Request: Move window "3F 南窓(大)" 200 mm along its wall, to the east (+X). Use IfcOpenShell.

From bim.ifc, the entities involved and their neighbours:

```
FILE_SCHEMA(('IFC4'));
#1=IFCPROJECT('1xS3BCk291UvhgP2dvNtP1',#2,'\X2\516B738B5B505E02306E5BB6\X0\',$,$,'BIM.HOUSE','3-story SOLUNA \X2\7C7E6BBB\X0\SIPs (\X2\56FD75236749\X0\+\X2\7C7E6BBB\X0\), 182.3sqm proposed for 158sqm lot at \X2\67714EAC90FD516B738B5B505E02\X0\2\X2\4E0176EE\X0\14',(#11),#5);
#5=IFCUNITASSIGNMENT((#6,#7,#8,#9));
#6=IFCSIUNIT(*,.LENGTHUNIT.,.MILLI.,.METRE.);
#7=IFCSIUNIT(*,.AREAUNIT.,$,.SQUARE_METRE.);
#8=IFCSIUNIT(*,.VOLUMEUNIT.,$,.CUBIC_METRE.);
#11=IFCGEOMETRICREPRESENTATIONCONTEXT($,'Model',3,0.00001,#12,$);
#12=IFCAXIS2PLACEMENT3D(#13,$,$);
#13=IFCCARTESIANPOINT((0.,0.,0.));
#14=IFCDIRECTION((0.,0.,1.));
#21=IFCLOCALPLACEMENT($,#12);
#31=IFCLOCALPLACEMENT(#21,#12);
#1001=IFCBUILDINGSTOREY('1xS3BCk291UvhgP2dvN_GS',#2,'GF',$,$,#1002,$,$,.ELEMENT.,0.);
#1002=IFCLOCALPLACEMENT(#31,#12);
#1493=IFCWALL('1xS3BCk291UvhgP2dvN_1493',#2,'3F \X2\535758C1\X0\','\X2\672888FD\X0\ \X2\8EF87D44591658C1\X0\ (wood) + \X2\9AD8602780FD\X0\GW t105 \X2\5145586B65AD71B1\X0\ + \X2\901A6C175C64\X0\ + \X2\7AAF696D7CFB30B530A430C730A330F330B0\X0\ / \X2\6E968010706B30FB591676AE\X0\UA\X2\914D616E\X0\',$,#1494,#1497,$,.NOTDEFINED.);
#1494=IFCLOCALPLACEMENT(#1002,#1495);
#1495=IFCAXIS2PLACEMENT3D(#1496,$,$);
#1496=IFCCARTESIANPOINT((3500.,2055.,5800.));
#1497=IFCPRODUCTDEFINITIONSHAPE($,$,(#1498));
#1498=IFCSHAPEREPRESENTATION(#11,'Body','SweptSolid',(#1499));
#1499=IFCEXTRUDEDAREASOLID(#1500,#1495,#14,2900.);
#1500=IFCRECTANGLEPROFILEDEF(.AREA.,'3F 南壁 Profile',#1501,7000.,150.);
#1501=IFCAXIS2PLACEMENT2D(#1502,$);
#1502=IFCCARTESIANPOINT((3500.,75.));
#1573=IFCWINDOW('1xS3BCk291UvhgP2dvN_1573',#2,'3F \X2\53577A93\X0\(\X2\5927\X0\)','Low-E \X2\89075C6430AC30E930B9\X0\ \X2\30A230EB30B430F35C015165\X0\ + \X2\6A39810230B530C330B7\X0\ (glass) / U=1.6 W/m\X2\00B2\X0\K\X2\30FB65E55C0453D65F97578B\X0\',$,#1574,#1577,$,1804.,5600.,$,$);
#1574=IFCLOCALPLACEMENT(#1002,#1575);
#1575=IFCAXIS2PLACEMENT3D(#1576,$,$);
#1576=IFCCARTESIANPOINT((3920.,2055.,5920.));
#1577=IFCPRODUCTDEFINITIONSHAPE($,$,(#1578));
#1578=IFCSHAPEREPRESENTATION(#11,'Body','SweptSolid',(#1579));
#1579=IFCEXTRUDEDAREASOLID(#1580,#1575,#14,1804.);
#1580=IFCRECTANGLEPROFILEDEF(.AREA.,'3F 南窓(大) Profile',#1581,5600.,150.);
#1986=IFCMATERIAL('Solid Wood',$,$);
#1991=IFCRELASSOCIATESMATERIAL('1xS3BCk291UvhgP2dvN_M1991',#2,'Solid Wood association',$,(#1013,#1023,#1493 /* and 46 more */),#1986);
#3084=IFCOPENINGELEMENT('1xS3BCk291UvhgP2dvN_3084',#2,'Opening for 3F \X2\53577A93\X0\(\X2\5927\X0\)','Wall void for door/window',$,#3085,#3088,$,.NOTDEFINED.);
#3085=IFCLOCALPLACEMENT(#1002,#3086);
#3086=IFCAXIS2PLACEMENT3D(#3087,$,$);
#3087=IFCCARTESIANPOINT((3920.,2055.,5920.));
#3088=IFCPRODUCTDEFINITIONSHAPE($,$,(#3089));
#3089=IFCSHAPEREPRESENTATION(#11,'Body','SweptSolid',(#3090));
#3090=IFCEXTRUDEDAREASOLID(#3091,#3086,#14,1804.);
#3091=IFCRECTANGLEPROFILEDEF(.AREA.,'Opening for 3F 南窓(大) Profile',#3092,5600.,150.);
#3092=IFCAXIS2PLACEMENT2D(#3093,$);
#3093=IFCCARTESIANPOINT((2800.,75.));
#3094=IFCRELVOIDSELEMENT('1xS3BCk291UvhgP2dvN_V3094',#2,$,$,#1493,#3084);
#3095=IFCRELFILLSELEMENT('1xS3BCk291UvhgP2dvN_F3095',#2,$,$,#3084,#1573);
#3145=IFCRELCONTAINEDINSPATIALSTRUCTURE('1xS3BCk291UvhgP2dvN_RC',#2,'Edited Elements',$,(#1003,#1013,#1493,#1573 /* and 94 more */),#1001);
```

```python
import ifcopenshell
import ifcopenshell.api.geometry
import ifcopenshell.util.placement
import ifcopenshell.util.unit

model = ifcopenshell.open("bim.ifc")
unit_scale = ifcopenshell.util.unit.calculate_unit_scale(model)

window = model.by_id(1573)
opening = window.FillsVoids[0].RelatingOpeningElement
wall = opening.VoidsElements[0].RelatingBuildingElement

wall_matrix = ifcopenshell.util.placement.get_local_placement(wall.ObjectPlacement)
shift = wall_matrix[:3, 0] * 0.2 / unit_scale
before = ifcopenshell.util.placement.get_local_placement(window.ObjectPlacement)[:3, 3].copy()

# The window is not placed relative to its opening, so move both.
for product in (opening, window):
    matrix = ifcopenshell.util.placement.get_local_placement(product.ObjectPlacement)
    matrix[:3, 3] += shift
    ifcopenshell.api.geometry.edit_object_placement(model, product=product, matrix=matrix, is_si=False)

after = ifcopenshell.util.placement.get_local_placement(window.ObjectPlacement)[:3, 3]
print("window moved by", (after - before).round(3) + 0.0)

model.write("bim_v2.ifc")
```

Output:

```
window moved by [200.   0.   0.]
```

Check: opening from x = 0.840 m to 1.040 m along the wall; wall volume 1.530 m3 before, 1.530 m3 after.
